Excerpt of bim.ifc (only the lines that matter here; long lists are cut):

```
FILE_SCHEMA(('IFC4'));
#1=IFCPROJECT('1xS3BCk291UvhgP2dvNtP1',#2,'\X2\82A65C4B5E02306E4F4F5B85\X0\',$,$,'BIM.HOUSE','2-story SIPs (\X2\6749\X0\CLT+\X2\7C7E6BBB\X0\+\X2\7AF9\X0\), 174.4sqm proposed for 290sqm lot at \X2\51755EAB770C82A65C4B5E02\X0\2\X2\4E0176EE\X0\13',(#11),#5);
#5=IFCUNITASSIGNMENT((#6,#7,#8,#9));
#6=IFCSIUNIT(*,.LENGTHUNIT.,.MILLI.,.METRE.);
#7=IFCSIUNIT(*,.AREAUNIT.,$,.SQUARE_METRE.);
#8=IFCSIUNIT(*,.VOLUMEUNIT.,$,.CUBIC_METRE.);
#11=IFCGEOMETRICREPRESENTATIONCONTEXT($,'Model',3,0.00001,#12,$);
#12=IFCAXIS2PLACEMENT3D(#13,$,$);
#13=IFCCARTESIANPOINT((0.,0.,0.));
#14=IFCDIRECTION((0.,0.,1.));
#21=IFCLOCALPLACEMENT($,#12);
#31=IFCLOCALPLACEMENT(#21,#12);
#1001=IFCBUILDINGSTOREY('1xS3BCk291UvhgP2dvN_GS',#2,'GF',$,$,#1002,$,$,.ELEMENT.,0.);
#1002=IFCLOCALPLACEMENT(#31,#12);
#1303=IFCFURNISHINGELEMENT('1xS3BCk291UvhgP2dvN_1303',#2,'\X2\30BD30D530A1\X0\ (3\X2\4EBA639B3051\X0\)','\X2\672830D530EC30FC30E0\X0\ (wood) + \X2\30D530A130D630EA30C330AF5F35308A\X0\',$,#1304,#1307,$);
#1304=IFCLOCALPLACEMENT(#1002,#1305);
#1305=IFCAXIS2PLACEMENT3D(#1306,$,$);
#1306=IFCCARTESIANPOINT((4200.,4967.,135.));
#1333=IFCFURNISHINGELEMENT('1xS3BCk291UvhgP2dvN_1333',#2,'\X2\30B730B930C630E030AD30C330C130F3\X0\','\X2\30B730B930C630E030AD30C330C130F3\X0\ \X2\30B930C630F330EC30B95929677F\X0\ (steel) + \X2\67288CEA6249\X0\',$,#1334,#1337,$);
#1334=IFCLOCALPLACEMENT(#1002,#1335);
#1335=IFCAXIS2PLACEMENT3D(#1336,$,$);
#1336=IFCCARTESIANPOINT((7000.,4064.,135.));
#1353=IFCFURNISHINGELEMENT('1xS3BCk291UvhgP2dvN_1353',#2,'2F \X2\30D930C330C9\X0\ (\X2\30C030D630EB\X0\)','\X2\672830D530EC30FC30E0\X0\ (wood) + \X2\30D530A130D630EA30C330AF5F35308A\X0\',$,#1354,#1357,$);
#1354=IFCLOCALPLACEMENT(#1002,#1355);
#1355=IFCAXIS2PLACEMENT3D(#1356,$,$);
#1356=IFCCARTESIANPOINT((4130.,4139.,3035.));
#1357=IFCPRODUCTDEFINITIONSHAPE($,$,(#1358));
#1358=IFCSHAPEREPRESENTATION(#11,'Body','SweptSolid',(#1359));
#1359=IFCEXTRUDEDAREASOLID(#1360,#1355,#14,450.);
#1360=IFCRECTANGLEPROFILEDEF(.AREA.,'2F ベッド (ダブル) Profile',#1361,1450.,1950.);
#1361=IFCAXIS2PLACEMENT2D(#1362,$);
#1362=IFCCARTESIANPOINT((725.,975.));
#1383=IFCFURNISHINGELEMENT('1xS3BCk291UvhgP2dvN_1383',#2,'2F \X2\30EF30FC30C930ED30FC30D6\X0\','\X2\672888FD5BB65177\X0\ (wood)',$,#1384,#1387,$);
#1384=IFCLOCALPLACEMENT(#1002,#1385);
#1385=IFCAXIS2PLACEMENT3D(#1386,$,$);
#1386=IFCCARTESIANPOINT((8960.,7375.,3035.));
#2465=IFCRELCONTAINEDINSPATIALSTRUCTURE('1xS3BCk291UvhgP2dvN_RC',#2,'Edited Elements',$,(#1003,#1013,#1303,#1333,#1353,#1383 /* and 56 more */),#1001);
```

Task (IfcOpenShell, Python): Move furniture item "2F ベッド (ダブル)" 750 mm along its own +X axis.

```python
import ifcopenshell
import ifcopenshell.api.geometry
import ifcopenshell.util.placement
import ifcopenshell.util.unit

model = ifcopenshell.open("bim.ifc")
unit_scale = ifcopenshell.util.unit.calculate_unit_scale(model)

item = model.by_id(1353)
matrix = ifcopenshell.util.placement.get_local_placement(item.ObjectPlacement)
matrix[:3, 3] += matrix[:3, 0] * 0.75 / unit_scale
ifcopenshell.api.geometry.edit_object_placement(model, product=item, matrix=matrix, is_si=False)

print(ifcopenshell.util.placement.get_local_placement(item.ObjectPlacement).round(3) + 0.0)

model.write("bim-out.ifc")
```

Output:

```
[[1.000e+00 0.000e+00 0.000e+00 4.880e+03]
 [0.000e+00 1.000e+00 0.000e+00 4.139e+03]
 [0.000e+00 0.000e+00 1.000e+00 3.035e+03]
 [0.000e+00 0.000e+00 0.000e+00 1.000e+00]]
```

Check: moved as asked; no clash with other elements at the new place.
